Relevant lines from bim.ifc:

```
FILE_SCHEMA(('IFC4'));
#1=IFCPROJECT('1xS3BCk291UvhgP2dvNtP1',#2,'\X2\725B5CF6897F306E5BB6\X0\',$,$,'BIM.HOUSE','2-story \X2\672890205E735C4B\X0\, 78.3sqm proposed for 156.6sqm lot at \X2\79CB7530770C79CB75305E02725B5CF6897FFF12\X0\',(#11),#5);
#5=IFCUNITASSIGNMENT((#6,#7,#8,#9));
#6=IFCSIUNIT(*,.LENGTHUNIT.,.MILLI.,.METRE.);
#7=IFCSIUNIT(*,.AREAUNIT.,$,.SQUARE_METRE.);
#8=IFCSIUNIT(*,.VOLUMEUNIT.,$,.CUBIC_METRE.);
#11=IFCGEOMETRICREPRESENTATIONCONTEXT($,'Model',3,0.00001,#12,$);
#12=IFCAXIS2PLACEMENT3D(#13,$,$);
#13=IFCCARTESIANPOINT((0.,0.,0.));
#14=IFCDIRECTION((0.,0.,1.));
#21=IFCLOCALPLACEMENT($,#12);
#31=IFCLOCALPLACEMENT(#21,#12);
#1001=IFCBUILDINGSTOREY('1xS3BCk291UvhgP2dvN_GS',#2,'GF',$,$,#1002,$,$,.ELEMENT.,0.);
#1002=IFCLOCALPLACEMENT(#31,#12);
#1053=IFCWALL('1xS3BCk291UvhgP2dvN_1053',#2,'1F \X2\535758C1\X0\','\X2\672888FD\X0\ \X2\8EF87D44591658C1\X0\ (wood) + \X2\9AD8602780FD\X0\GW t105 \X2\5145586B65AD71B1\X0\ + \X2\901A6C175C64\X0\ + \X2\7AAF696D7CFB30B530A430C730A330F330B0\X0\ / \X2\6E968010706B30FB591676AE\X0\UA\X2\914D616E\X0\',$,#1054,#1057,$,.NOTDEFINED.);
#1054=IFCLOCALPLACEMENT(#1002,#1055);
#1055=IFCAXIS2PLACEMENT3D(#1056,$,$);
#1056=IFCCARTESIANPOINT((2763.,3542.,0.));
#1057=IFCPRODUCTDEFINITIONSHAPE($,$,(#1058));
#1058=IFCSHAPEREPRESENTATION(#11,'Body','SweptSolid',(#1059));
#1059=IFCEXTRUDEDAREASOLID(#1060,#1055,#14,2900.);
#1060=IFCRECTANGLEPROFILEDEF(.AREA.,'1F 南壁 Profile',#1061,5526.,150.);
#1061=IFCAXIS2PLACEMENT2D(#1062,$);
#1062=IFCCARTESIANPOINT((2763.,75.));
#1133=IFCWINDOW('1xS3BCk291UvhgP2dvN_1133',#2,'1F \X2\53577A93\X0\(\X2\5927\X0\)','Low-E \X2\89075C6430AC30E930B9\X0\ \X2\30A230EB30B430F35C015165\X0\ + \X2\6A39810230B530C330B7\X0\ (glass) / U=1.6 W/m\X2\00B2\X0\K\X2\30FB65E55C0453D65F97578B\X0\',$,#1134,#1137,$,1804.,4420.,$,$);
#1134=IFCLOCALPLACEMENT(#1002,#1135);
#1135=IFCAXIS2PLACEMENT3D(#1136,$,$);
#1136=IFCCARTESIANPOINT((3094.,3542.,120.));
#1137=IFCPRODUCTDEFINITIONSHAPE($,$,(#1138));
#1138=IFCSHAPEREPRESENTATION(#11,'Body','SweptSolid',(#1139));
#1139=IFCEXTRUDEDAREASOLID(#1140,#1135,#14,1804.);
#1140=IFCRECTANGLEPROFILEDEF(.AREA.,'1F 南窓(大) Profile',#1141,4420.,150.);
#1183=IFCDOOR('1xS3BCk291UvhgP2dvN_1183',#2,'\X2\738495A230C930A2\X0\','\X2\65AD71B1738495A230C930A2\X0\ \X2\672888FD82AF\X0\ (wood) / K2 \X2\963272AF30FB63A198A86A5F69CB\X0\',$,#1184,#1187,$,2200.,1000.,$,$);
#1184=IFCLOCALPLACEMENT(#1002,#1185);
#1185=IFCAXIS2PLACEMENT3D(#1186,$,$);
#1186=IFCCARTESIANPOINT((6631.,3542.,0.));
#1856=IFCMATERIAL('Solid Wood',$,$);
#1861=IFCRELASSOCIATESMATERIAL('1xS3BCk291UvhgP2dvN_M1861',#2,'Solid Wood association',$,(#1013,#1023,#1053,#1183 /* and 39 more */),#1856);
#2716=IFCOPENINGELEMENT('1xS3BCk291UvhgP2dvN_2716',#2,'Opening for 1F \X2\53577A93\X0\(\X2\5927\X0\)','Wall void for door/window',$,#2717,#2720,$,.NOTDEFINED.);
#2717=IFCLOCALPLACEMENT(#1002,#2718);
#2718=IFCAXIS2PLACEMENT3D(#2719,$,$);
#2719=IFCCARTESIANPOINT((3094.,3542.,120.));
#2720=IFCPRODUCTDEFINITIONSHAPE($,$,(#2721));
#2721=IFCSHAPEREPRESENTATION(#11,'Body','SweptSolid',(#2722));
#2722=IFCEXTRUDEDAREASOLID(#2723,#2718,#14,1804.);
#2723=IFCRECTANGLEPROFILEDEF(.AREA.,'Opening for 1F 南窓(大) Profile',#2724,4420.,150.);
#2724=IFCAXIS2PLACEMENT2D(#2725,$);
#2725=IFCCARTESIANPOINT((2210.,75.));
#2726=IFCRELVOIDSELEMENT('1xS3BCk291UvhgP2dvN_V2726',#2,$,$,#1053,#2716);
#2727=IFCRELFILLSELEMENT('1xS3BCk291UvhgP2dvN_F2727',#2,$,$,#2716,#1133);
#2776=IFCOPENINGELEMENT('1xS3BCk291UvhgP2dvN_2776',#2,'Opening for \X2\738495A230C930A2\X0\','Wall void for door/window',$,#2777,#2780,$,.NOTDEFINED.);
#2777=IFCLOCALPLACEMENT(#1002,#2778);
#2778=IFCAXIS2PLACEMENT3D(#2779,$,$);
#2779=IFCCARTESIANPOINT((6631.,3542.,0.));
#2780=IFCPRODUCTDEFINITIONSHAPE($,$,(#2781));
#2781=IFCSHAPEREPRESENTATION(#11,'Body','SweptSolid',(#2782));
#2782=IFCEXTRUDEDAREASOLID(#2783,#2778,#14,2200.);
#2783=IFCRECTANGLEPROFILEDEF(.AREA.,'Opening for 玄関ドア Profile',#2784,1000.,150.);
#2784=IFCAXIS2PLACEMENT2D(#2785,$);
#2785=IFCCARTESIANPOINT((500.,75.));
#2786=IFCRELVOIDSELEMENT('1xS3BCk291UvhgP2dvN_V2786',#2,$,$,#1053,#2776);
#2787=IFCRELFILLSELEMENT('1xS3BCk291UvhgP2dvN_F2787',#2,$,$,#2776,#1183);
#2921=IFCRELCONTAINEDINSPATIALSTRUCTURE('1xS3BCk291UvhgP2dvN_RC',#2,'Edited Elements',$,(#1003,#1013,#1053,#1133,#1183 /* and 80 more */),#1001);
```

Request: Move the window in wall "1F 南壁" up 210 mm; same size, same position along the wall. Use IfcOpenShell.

```python
import numpy as np
import ifcopenshell
import ifcopenshell.api.geometry
import ifcopenshell.util.placement
import ifcopenshell.util.unit

model = ifcopenshell.open("bim.ifc")
unit_scale = ifcopenshell.util.unit.calculate_unit_scale(model)

window = model.by_guid("1xS3BCk291UvhgP2dvN_1133")
opening = window.FillsVoids[0].RelatingOpeningElement
dz = 210.0

shift = np.array([0.0, 0.0, dz])
# The window is not placed relative to its opening, so move both.
for product in (opening, window):
    matrix = ifcopenshell.util.placement.get_local_placement(product.ObjectPlacement)
    matrix[:3, 3] += shift
    ifcopenshell.api.geometry.edit_object_placement(model, product=product, matrix=matrix, is_si=False)

print(f"moved by {dz * unit_scale:+.3f} m")

model.write("bim_updated.ifc")
```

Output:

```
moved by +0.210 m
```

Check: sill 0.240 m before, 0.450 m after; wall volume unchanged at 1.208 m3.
